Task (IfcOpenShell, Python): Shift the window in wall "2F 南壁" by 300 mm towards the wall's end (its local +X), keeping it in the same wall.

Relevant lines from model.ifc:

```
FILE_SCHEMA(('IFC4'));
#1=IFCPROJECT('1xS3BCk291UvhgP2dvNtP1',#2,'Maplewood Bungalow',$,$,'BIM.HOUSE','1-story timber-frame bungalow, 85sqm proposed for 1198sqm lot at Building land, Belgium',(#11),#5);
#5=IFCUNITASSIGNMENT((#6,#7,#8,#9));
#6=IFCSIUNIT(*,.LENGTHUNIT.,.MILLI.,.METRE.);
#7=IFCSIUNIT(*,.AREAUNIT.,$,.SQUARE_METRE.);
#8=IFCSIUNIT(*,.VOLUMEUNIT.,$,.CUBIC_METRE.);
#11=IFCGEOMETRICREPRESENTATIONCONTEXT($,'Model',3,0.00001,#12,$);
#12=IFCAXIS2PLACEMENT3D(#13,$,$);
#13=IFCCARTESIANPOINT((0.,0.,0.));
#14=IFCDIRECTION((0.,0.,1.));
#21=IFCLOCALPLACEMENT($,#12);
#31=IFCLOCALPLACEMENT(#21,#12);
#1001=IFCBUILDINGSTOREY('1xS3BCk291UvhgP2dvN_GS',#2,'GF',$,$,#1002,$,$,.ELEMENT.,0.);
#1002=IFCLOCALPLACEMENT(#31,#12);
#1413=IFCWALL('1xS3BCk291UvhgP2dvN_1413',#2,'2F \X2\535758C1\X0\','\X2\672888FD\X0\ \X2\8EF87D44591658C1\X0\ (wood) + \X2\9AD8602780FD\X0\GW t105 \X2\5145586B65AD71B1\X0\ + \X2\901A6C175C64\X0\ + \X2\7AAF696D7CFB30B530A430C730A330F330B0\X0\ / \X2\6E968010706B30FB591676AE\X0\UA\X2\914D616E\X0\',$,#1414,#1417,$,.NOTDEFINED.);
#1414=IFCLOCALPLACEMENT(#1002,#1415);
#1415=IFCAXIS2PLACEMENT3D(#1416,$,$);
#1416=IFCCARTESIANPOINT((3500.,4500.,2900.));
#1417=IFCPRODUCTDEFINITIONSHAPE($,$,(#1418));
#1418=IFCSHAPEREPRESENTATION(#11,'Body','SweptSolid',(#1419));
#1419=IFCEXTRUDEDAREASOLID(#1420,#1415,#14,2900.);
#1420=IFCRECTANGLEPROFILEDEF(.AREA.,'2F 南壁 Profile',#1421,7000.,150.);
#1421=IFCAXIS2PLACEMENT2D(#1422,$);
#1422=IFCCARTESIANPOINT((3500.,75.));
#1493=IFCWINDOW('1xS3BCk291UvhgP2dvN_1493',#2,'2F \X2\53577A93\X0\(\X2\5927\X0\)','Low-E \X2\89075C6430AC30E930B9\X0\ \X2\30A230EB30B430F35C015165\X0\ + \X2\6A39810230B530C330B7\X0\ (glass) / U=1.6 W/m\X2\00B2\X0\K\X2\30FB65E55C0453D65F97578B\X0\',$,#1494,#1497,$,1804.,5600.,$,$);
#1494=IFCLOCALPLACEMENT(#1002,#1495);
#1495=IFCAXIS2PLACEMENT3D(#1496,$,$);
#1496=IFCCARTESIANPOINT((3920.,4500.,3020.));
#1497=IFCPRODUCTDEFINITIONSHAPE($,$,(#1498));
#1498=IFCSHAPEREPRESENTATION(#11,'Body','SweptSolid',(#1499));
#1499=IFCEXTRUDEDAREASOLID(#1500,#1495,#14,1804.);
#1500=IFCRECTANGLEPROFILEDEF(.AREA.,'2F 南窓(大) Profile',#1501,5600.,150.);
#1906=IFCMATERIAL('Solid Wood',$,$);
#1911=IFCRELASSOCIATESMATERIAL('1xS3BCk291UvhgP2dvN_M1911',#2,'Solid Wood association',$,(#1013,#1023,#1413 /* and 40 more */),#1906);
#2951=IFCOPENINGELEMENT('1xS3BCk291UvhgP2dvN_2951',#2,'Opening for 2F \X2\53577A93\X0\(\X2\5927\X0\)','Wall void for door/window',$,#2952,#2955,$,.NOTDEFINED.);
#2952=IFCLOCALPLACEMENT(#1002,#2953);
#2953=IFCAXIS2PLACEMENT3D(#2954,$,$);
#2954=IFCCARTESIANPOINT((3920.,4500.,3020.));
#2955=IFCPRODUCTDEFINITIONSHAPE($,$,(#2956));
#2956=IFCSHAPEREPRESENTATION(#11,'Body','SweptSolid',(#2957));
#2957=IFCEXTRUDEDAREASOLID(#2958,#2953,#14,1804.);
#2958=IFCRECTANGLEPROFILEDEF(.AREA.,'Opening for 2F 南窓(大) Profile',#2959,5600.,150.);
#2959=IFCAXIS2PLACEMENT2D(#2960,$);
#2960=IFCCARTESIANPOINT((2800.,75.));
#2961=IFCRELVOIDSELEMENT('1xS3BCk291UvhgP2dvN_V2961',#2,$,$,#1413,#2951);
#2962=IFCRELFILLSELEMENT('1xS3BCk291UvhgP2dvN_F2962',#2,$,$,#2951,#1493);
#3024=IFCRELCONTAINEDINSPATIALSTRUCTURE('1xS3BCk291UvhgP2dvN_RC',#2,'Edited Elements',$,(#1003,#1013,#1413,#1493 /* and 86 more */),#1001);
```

```python
import ifcopenshell
import ifcopenshell.api.geometry
import ifcopenshell.util.placement

model = ifcopenshell.open("model.ifc")

window = model.by_guid("1xS3BCk291UvhgP2dvN_1493")
opening = window.FillsVoids[0].RelatingOpeningElement
wall = opening.VoidsElements[0].RelatingBuildingElement

wall_matrix = ifcopenshell.util.placement.get_local_placement(wall.ObjectPlacement)
shift = wall_matrix[:3, 0] * 300.0
before = ifcopenshell.util.placement.get_local_placement(window.ObjectPlacement)[:3, 3].copy()

# The window is not placed relative to its opening, so move both.
for product in (opening, window):
    matrix = ifcopenshell.util.placement.get_local_placement(product.ObjectPlacement)
    matrix[:3, 3] += shift
    ifcopenshell.api.geometry.edit_object_placement(model, product=product, matrix=matrix, is_si=False)

after = ifcopenshell.util.placement.get_local_placement(window.ObjectPlacement)[:3, 3]
print("window moved by", (after - before).round(3) + 0.0)

model.write("model_v2.ifc")
```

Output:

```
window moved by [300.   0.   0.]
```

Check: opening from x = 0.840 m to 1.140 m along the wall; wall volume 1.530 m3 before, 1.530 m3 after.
